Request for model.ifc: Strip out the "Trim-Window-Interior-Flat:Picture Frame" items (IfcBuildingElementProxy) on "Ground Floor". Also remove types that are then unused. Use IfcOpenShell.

First a look at what the model holds.

```python
import ifcopenshell
import ifcopenshell.util.element

model = ifcopenshell.open("model.ifc")
print(model.schema)
storey = next(s for s in model.by_type("IfcBuildingStorey") if s.Name == "Ground Floor")
proxies = [e for e in ifcopenshell.util.element.get_decomposition(storey) if e.is_a("IfcBuildingElementProxy")]
seen = {}
for e in proxies:
    element_type = ifcopenshell.util.element.get_type(e)
    name = element_type.Name if element_type not in (None, e) else None
    seen[name] = seen.get(name, 0) + 1
for name, count in sorted(seen.items(), key=str):
    print(count, "x", name)
```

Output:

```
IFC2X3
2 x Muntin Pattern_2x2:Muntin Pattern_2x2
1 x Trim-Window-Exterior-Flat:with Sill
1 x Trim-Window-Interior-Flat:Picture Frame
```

```python
import ifcopenshell
import ifcopenshell.api.root
import ifcopenshell.util.element

model = ifcopenshell.open("model.ifc")

storey = next(s for s in model.by_type("IfcBuildingStorey") if s.Name == "Ground Floor")
proxies = [e for e in ifcopenshell.util.element.get_decomposition(storey) if e.is_a("IfcBuildingElementProxy")]
targets = [e for e in proxies if (t := ifcopenshell.util.element.get_type(e)) not in (None, e) and t.Name == "Trim-Window-Interior-Flat:Picture Frame"]
types = {ifcopenshell.util.element.get_type(e) for e in targets} - {None, *targets}

for e in targets:
    ifcopenshell.api.root.remove_product(model, product=e)
print(len(targets), "removed")

unused = [t for t in types if not ifcopenshell.util.element.get_types(t)]
for t in unused:
    ifcopenshell.api.root.remove_product(model, product=t)
print(len(unused), "unused types removed")

model.write("model_edited.ifc")
```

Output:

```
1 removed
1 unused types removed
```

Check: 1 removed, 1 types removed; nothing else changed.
